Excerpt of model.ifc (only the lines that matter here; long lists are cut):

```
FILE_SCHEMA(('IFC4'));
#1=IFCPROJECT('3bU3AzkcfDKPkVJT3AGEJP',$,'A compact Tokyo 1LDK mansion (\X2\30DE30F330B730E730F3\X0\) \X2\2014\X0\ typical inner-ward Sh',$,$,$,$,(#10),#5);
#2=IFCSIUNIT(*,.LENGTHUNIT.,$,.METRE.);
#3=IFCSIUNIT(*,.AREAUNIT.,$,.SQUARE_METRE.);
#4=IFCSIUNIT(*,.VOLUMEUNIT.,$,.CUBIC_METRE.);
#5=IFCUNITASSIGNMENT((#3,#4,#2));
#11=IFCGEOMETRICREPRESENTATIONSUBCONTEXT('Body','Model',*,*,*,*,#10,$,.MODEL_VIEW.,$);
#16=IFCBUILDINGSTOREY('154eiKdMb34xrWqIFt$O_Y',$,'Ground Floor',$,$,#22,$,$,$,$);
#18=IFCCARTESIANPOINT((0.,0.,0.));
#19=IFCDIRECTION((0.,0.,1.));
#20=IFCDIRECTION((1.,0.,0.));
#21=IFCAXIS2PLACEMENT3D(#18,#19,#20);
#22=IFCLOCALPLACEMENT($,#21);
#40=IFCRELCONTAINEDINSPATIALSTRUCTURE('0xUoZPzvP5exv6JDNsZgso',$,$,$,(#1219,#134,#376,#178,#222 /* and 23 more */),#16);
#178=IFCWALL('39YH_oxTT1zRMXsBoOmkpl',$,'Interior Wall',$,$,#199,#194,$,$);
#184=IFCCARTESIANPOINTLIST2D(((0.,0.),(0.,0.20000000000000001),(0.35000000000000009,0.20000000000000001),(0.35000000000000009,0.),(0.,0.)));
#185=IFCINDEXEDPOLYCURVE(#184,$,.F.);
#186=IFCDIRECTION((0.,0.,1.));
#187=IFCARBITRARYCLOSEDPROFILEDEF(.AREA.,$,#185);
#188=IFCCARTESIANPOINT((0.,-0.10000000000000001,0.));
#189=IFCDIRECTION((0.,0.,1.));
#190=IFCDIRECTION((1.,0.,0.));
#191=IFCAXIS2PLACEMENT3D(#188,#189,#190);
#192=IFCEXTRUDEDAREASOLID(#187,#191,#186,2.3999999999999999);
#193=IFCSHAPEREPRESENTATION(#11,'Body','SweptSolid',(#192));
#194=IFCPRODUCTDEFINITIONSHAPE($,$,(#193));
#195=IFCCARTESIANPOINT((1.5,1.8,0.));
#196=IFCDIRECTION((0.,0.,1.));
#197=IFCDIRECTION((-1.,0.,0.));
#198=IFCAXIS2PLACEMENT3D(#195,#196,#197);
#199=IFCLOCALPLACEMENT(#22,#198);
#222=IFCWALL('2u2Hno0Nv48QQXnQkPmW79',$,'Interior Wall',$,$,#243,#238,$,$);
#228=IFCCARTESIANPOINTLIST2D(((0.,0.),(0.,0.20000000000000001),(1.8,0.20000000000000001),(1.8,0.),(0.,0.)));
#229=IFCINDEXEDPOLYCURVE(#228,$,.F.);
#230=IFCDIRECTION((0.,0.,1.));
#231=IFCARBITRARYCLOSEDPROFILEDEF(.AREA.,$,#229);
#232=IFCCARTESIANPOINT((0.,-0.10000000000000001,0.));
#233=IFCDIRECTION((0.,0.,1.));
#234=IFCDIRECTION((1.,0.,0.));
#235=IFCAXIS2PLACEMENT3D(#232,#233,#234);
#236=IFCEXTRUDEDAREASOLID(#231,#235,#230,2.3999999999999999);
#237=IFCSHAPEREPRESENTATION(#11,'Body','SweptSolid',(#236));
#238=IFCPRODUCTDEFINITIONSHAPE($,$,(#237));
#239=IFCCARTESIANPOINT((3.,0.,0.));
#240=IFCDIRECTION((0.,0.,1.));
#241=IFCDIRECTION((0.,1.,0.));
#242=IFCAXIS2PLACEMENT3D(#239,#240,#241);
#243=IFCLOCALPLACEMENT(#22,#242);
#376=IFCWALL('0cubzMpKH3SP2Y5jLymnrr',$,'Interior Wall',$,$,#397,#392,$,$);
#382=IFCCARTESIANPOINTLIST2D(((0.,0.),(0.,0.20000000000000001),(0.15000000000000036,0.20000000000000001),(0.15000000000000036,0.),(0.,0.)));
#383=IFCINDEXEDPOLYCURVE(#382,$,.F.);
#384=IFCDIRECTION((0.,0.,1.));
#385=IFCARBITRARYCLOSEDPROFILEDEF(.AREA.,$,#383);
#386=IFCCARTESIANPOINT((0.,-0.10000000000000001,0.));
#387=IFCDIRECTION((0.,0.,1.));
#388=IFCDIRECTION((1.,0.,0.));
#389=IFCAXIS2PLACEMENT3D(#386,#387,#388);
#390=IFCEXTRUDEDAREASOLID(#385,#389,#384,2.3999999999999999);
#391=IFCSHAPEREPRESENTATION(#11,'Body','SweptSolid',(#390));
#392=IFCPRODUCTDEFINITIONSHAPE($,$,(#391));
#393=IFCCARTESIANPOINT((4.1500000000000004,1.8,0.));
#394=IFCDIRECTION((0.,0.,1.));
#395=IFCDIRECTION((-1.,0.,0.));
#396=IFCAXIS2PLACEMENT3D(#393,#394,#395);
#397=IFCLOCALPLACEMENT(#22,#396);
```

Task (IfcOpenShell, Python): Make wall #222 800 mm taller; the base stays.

```python
import ifcopenshell
import ifcopenshell.geom
import ifcopenshell.util.representation
import ifcopenshell.util.shape
import ifcopenshell.util.unit

model = ifcopenshell.open("model.ifc")
unit_scale = ifcopenshell.util.unit.calculate_unit_scale(model)
settings = ifcopenshell.geom.settings()


def volume(element):
    """Net volume in cubic metres, openings subtracted."""
    shape = ifcopenshell.geom.create_shape(settings, element)
    return ifcopenshell.util.shape.get_volume(shape.geometry)


wall = model.by_id(222)
before = volume(wall)

body = ifcopenshell.util.representation.get_representation(wall, "Model", "Body")
solid = body.Items[0]
old_height = solid.Depth
solid.Depth += 0.8 / unit_scale
after = volume(wall)

print(f"height {old_height:g} -> {solid.Depth:g}, volume {before:.3f} -> {after:.3f} m3")

model.write("model_updated.ifc")
```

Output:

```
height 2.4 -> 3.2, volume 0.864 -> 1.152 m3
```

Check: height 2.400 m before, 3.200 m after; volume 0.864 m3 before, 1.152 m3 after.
